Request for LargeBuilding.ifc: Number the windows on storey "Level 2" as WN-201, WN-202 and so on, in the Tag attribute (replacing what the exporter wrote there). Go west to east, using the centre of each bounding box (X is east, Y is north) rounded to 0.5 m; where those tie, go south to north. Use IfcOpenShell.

First a look at what the model holds.

```python
import ifcopenshell
import ifcopenshell.util.element
import ifcopenshell.util.placement

model = ifcopenshell.open("LargeBuilding.ifc")
print(model.schema)
storey = next(s for s in model.by_type("IfcBuildingStorey") if s.Name == "Level 2")
windows = [e for e in ifcopenshell.util.element.get_decomposition(storey) if e.is_a("IfcWindow")]
for e in sorted(windows, key=lambda e: e.id()):
    origin = ifcopenshell.util.placement.get_local_placement(e.ObjectPlacement)[:3, 3]
    print(e.id(), e.Tag, e.Name, origin.round(2) + 0.0, sep=" | ")
```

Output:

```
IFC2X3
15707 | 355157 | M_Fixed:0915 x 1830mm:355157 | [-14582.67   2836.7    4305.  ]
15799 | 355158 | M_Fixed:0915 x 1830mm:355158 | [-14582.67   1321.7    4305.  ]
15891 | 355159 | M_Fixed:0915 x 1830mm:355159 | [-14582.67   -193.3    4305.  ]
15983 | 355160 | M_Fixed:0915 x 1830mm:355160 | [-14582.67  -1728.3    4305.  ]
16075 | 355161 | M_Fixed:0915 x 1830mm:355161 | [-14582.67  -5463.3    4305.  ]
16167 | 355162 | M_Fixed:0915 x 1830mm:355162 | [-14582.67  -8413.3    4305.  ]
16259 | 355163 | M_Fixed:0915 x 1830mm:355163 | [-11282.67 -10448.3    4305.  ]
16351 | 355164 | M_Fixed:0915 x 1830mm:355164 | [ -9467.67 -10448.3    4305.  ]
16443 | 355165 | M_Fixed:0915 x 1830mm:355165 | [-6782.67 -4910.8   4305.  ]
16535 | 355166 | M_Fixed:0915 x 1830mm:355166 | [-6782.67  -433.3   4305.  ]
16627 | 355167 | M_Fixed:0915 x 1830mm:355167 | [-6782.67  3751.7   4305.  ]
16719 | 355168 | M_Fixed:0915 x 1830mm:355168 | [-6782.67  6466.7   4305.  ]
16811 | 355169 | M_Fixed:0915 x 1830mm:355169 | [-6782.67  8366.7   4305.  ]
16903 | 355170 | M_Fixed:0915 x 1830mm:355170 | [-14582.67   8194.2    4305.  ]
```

```python
import ifcopenshell
import ifcopenshell.geom
import ifcopenshell.util.element
import ifcopenshell.util.shape

model = ifcopenshell.open("LargeBuilding.ifc")
settings = ifcopenshell.geom.settings()
settings.set("use-world-coords", True)


def centre(element):
    shape = ifcopenshell.geom.create_shape(settings, element)
    return ifcopenshell.util.shape.get_bbox_centroid(shape.geometry)


storey = next(s for s in model.by_type("IfcBuildingStorey") if s.Name == "Level 2")
windows = [e for e in ifcopenshell.util.element.get_decomposition(storey) if e.is_a("IfcWindow")]

# Insertion points can sit at a corner or the storey origin, so sort by the geometry (in metres).
centres = {e: centre(e) for e in windows}
windows.sort(key=lambda e: (round(centres[e][0] / 0.5), centres[e][1]))

for i, e in enumerate(windows, start=1):
    number = f"WN-2{i:02d}"
    e.Tag = number
    print(e.id(), number)

model.write("LargeBuilding-out.ifc")
```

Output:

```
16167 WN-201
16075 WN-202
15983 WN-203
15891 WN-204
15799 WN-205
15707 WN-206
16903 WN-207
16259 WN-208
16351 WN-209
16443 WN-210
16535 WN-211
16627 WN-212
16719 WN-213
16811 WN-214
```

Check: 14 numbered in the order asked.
